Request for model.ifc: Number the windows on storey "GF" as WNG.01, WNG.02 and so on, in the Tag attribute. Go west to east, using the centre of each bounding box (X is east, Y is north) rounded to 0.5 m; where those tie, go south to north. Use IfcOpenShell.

First a look at what the model holds.

```python
import ifcopenshell
import ifcopenshell.util.element
import ifcopenshell.util.placement

model = ifcopenshell.open("model.ifc")
print(model.schema)
storey = next(s for s in model.by_type("IfcBuildingStorey") if s.Name == "GF")
windows = [e for e in ifcopenshell.util.element.get_decomposition(storey) if e.is_a("IfcWindow")]
for e in sorted(windows, key=lambda e: e.id()):
    origin = ifcopenshell.util.placement.get_local_placement(e.ObjectPlacement)[:3, 3]
    print(e.id(), e.Tag, e.Name, origin.round(2) + 0.0, sep=" | ")
```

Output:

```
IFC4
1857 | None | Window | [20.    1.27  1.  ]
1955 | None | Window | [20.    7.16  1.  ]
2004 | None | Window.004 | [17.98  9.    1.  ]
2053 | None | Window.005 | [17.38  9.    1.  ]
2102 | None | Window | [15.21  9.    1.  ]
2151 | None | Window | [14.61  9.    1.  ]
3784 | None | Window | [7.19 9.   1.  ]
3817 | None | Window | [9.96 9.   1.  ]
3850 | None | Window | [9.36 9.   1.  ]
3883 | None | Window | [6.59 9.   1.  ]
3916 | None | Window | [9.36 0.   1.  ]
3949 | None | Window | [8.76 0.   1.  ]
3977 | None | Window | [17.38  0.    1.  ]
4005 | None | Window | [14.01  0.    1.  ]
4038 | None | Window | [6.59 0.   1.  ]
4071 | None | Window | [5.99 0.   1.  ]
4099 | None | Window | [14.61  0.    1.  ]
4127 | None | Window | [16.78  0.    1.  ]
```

```python
import ifcopenshell
import ifcopenshell.geom
import ifcopenshell.util.element
import ifcopenshell.util.shape

model = ifcopenshell.open("model.ifc")
settings = ifcopenshell.geom.settings()
settings.set("use-world-coords", True)


def centre(element):
    shape = ifcopenshell.geom.create_shape(settings, element)
    return ifcopenshell.util.shape.get_bbox_centroid(shape.geometry)


storey = next(s for s in model.by_type("IfcBuildingStorey") if s.Name == "GF")
windows = [e for e in ifcopenshell.util.element.get_decomposition(storey) if e.is_a("IfcWindow")]

# Insertion points can sit at a corner or the storey origin, so sort by the geometry (in metres).
centres = {e: centre(e) for e in windows}
windows.sort(key=lambda e: (round(centres[e][0] / 0.5), centres[e][1]))

for i, e in enumerate(windows, start=1):
    number = f"WNG.{i:02d}"
    e.Tag = number
    print(e.id(), number)

model.write("model_edited.ifc")
```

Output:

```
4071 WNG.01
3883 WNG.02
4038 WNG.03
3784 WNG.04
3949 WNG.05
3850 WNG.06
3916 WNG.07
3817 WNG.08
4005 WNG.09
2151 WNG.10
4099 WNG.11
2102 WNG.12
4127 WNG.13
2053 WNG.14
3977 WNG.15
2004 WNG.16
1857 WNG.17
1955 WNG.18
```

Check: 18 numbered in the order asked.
